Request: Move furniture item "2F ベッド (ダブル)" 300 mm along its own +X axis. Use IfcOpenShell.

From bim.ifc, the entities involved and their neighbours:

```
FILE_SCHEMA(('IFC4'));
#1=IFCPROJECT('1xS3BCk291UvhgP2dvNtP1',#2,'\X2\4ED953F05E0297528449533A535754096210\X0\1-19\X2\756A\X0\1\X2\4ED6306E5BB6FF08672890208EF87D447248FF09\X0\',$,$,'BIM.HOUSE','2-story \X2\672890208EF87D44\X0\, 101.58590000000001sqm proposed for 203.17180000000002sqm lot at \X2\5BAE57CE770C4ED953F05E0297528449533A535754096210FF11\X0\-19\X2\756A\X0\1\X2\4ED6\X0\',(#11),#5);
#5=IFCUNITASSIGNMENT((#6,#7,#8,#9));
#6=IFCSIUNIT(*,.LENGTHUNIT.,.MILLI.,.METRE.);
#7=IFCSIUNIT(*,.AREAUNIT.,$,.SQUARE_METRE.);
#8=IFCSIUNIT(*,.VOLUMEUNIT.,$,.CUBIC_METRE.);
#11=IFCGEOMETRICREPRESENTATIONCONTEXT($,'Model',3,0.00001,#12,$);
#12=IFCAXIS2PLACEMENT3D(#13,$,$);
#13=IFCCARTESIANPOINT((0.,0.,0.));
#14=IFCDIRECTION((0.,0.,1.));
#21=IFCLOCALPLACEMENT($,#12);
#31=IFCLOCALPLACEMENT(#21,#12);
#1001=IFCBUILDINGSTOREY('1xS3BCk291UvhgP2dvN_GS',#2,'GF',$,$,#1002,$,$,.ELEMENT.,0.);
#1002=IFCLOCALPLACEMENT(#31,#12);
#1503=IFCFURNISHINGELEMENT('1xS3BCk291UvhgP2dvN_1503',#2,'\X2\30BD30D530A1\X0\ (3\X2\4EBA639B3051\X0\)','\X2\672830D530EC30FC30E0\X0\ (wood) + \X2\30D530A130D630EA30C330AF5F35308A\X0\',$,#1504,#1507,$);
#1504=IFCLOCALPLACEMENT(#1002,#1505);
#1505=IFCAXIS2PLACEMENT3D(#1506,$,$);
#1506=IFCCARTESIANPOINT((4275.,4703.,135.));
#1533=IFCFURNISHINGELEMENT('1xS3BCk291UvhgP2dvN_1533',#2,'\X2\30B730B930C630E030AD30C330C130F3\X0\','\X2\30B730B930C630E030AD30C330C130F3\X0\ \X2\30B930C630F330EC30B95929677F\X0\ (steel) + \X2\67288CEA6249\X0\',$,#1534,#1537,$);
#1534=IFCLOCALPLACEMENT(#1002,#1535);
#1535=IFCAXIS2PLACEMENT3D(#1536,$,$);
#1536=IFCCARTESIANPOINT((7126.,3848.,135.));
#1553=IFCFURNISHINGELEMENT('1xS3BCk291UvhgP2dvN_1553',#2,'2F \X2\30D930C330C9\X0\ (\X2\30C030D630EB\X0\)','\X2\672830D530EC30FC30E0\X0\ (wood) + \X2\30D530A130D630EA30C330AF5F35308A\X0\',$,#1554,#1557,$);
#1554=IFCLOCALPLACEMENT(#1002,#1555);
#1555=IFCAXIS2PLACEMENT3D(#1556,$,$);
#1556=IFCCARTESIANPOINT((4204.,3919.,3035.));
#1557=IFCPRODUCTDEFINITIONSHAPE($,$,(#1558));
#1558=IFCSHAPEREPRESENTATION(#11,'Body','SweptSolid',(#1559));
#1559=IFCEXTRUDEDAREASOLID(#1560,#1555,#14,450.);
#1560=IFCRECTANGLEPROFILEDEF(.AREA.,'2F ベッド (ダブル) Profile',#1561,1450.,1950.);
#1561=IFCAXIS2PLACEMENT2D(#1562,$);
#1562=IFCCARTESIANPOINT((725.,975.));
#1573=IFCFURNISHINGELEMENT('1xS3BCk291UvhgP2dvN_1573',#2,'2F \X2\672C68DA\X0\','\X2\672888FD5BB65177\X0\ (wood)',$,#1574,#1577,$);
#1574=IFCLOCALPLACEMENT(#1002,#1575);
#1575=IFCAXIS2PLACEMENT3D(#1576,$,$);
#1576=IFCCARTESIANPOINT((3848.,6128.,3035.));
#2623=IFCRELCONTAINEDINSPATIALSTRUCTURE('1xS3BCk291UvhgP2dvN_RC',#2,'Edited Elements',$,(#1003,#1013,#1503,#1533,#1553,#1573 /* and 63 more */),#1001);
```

```python
import ifcopenshell
import ifcopenshell.api.geometry
import ifcopenshell.util.placement

model = ifcopenshell.open("bim.ifc")

item = model.by_id(1553)
matrix = ifcopenshell.util.placement.get_local_placement(item.ObjectPlacement)
matrix[:3, 3] += matrix[:3, 0] * 300.0
ifcopenshell.api.geometry.edit_object_placement(model, product=item, matrix=matrix, is_si=False)

print(ifcopenshell.util.placement.get_local_placement(item.ObjectPlacement).round(3) + 0.0)

model.write("bim-out.ifc")
```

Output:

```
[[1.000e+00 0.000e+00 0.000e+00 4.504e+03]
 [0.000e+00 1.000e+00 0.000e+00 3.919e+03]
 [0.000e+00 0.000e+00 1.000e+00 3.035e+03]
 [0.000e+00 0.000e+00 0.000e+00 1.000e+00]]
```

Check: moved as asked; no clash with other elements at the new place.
